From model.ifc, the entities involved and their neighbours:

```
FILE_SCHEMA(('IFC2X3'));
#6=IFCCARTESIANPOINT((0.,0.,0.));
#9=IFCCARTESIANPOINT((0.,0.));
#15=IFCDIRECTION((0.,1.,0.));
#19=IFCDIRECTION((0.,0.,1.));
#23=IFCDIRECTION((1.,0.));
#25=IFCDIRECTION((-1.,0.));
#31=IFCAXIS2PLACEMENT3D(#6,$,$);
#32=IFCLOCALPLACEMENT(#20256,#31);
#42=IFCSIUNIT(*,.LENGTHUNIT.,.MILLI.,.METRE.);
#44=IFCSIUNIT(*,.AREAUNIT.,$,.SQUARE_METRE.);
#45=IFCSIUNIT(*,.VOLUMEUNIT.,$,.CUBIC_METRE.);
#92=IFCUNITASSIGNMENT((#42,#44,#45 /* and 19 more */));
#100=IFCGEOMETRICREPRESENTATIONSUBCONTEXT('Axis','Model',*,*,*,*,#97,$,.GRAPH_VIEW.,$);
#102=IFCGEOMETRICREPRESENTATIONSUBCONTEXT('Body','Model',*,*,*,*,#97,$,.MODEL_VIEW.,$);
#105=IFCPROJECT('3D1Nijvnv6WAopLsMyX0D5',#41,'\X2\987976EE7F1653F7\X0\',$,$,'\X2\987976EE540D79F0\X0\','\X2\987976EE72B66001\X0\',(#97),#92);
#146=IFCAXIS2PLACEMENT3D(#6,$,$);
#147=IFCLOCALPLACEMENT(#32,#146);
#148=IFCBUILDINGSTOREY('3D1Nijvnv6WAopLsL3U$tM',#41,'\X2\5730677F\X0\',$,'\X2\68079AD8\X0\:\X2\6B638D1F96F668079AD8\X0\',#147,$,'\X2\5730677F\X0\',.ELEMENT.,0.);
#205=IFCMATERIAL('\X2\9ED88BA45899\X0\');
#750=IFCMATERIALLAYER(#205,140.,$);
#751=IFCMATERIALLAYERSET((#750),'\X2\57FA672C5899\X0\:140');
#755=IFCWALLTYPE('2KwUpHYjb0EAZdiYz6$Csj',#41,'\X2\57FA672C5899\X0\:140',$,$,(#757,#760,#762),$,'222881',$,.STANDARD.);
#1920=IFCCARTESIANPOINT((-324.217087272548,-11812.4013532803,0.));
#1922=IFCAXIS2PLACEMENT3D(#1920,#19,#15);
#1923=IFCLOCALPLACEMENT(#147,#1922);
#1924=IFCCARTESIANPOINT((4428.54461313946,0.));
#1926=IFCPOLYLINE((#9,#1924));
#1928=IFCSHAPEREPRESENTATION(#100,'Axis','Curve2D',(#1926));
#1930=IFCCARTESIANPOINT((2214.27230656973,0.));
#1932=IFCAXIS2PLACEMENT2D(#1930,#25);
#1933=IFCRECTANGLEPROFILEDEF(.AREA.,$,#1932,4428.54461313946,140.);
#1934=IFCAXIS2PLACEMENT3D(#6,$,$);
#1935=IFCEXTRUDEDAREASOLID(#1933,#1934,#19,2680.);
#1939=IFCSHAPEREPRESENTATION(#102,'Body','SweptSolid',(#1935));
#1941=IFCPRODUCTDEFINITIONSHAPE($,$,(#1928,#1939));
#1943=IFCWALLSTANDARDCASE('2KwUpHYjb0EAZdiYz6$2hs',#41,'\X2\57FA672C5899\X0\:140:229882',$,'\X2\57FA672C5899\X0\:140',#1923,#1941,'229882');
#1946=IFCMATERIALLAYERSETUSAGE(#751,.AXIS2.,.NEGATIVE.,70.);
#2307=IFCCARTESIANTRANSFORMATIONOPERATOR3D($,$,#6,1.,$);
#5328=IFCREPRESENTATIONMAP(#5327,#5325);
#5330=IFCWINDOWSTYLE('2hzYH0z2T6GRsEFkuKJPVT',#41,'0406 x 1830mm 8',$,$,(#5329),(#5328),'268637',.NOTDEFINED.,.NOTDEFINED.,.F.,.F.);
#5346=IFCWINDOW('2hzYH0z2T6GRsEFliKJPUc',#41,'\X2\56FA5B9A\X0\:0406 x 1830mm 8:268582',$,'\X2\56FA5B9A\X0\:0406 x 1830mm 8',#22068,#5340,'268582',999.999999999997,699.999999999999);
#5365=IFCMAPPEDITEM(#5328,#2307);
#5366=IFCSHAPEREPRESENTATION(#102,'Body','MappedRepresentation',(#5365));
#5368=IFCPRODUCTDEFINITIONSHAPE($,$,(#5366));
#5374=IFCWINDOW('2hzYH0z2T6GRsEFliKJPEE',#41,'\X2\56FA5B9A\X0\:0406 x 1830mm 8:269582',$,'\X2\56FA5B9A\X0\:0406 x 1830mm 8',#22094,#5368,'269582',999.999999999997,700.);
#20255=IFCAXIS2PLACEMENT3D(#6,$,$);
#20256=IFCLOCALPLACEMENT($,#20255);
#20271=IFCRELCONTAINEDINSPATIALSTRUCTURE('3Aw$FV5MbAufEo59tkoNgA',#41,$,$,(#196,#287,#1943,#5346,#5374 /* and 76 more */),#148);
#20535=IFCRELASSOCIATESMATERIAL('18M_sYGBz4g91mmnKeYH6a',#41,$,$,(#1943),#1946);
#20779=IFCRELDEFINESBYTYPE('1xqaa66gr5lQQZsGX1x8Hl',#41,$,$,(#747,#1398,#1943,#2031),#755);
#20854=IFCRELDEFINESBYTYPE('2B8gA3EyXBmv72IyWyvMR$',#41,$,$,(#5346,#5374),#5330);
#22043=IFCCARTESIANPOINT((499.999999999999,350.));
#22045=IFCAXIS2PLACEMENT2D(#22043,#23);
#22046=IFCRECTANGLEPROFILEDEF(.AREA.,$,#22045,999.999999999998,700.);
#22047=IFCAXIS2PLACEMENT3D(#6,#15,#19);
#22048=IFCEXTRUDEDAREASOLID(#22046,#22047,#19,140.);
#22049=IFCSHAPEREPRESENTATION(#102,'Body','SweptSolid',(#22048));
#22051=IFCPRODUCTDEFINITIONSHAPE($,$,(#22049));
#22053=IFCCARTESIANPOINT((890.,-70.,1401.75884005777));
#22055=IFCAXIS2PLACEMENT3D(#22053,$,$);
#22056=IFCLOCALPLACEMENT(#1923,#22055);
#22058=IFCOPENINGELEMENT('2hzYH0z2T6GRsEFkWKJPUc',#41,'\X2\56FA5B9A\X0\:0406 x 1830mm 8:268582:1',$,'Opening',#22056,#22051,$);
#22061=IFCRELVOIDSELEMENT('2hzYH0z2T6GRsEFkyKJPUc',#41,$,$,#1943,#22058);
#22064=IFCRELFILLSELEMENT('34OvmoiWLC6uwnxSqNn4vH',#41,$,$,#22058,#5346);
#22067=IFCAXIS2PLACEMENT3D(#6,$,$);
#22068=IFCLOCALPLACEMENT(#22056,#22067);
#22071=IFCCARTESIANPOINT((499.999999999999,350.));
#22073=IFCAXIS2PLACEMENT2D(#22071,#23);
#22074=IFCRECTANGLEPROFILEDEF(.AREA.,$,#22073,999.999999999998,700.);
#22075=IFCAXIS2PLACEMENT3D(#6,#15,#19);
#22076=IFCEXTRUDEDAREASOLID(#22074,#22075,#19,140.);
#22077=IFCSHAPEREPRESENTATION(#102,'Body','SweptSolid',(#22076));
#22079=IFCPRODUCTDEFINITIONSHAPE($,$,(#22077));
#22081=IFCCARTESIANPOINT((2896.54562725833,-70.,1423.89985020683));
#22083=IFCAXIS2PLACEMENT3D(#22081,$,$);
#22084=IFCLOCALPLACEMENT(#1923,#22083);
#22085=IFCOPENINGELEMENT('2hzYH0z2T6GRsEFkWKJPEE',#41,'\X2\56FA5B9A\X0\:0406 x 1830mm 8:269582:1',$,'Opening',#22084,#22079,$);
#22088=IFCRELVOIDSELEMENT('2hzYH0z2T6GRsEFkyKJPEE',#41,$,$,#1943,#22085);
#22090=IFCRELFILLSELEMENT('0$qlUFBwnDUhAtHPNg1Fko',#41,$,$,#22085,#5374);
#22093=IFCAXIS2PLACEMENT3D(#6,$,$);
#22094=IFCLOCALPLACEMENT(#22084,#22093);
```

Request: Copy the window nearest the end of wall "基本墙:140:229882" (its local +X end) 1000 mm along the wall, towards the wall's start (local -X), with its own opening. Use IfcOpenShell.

```python
import ifcopenshell
import ifcopenshell.api.feature
import ifcopenshell.api.geometry
import ifcopenshell.api.root
import ifcopenshell.geom
import ifcopenshell.util.element
import ifcopenshell.util.placement
import ifcopenshell.util.shape

model = ifcopenshell.open("model.ifc")
settings = ifcopenshell.geom.settings()


def volume(element):
    """Net volume in cubic metres, openings subtracted."""
    shape = ifcopenshell.geom.create_shape(settings, element)
    return ifcopenshell.util.shape.get_volume(shape.geometry)


def reuse_history(source, copy):
    """copy_class also copies each property set's owner history, people and application; keep the originals."""
    for rel in copy.IsDefinedBy:
        if rel.is_a("IfcRelDefinesByProperties") and (history := rel.RelatingPropertyDefinition.OwnerHistory):
            rel.RelatingPropertyDefinition.OwnerHistory = source.OwnerHistory
            ifcopenshell.util.element.remove_deep2(model, history)


window = model.by_id(5374)
opening = window.FillsVoids[0].RelatingOpeningElement
wall = opening.VoidsElements[0].RelatingBuildingElement
before = volume(wall)
shift = ifcopenshell.util.placement.get_local_placement(wall.ObjectPlacement)[:3, 0] * -1000.0

# copy_class copies the void relationship, type, container and properties, but no geometry.
new_opening = ifcopenshell.api.root.copy_class(model, product=opening)
new_opening.Representation = ifcopenshell.util.element.copy_deep(
    model, opening.Representation, exclude=["IfcGeometricRepresentationContext", "IfcRepresentationMap"]
)
new_opening.Name = "固定:0406 x 1830mm 8"
new_window = ifcopenshell.api.root.copy_class(model, product=window)
new_window.Representation = ifcopenshell.util.element.copy_deep(
    model, window.Representation, exclude=["IfcGeometricRepresentationContext", "IfcRepresentationMap"]
)
new_window.Name = "固定:0406 x 1830mm 8"
new_window.Tag = None
reuse_history(window, new_window)
fills = ifcopenshell.api.feature.add_filling(model, opening=new_opening, element=new_window)
fills.OwnerHistory = new_window.OwnerHistory  # required in IFC2X3

for old, new in ((opening, new_opening), (window, new_window)):
    matrix = ifcopenshell.util.placement.get_local_placement(old.ObjectPlacement)
    matrix[:3, 3] += shift
    ifcopenshell.api.geometry.edit_object_placement(model, product=new, matrix=matrix, is_si=False)

after = volume(wall)

print(f"wall volume {before:.3f} -> {after:.3f} m3")

model.write("model_rev.ifc")
```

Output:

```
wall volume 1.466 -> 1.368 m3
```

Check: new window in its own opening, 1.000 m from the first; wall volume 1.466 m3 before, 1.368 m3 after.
